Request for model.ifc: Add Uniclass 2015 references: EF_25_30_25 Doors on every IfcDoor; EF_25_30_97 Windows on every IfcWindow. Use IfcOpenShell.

First a look at what the model holds.

```python
import ifcopenshell

model = ifcopenshell.open("model.ifc")
print(model.schema)
print("classifications:", [c.Name for c in model.by_type("IfcClassification")])
for ifc_class in ("IfcDoor", "IfcRoof", "IfcStair", "IfcWall", "IfcWindow"):
    print(ifc_class, len(model.by_type(ifc_class)))
```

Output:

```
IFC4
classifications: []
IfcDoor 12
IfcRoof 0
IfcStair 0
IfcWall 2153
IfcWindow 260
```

```python
import ifcopenshell
import ifcopenshell.api.classification

model = ifcopenshell.open("model.ifc")

system = ifcopenshell.api.classification.add_classification(model, classification="Uniclass 2015")

codes = {
    "IfcDoor": ("EF_25_30_25", "Doors"),
    "IfcWindow": ("EF_25_30_97", "Windows"),
}
for ifc_class, (code, name) in codes.items():
    products = model.by_type(ifc_class)
    ifcopenshell.api.classification.add_reference(
        model, products=products, classification=system, identification=code, name=name
    )
    print(code, len(products))

model.write("model_rev.ifc")
```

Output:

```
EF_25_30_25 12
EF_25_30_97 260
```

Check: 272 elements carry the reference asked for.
